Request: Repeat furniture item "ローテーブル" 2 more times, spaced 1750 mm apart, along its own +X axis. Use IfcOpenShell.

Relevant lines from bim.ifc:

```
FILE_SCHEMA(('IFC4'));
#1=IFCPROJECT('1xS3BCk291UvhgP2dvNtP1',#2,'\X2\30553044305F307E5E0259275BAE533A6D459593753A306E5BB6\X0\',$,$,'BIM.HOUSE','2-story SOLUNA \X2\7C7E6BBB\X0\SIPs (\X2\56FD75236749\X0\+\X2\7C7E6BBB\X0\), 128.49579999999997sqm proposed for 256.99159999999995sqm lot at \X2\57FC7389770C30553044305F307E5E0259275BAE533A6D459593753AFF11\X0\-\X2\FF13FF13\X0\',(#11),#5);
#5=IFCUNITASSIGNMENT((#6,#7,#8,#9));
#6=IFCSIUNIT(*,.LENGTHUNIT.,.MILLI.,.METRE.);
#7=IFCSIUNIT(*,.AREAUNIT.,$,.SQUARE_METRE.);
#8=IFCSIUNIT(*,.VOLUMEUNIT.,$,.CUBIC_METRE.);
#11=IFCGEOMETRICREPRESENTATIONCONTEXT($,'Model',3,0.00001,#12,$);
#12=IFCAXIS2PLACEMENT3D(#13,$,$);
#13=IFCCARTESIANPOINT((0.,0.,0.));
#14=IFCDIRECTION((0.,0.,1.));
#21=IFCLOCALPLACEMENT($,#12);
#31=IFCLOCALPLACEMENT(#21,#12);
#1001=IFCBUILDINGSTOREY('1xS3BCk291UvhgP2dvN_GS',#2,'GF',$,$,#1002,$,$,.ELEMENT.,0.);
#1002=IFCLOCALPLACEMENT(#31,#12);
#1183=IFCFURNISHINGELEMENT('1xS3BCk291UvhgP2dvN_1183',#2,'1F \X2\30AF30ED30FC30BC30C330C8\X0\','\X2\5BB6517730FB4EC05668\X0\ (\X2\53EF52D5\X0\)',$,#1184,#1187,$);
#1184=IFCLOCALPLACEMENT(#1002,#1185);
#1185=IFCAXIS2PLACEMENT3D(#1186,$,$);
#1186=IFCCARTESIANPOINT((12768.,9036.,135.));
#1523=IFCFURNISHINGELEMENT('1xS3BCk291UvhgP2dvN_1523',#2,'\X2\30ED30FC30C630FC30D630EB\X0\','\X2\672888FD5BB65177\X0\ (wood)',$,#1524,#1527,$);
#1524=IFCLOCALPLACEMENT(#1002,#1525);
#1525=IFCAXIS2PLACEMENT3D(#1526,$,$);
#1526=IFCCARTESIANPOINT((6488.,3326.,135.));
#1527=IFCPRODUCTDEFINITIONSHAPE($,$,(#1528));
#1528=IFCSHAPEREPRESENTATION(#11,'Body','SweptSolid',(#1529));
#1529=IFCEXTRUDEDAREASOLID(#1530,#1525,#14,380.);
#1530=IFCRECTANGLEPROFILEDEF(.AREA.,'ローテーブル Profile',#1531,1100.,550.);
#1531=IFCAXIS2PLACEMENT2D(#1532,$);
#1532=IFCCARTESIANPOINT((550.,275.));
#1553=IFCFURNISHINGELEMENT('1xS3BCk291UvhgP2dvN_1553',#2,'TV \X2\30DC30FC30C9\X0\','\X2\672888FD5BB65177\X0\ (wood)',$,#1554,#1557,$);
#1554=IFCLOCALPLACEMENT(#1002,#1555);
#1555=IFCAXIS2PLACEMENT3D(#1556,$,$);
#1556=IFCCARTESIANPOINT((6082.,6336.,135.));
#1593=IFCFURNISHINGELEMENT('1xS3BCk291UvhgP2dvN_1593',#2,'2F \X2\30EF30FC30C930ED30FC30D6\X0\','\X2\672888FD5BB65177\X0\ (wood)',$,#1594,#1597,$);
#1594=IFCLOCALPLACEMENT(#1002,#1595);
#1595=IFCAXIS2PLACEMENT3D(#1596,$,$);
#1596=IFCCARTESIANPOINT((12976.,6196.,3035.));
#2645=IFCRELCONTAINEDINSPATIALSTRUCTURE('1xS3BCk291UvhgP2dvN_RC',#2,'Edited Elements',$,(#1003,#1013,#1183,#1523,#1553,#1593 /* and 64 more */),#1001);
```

```python
import ifcopenshell
import ifcopenshell.api.geometry
import ifcopenshell.api.root
import ifcopenshell.util.element
import ifcopenshell.util.placement

model = ifcopenshell.open("bim.ifc")


def reuse_history(source, copy):
    """copy_class also copies each property set's owner history, people and application; keep the originals."""
    for rel in copy.IsDefinedBy:
        if rel.is_a("IfcRelDefinesByProperties") and (history := rel.RelatingPropertyDefinition.OwnerHistory):
            rel.RelatingPropertyDefinition.OwnerHistory = source.OwnerHistory
            ifcopenshell.util.element.remove_deep2(model, history)


source = model.by_id(1523)
base = ifcopenshell.util.placement.get_local_placement(source.ObjectPlacement)
step = base[:3, 0] * 1750.0

for i in range(1, 3):
    copy = ifcopenshell.api.root.copy_class(model, product=source)
    copy.Representation = ifcopenshell.util.element.copy_deep(
        model, source.Representation, exclude=["IfcGeometricRepresentationContext", "IfcRepresentationMap"]
    )
    reuse_history(source, copy)
    matrix = base.copy()
    matrix[:3, 3] += i * step
    print("added at", matrix[:3, 3].round(3) + 0.0)
    ifcopenshell.api.geometry.edit_object_placement(model, product=copy, matrix=matrix, is_si=False)

model.write("bim_v2.ifc")
```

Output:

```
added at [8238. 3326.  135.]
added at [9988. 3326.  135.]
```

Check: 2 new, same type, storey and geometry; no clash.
